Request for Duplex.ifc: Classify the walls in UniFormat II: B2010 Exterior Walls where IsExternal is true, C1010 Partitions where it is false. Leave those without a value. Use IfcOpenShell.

First a look at what the model holds.

```python
import ifcopenshell
import ifcopenshell.util.element

model = ifcopenshell.open("Duplex.ifc")
print(model.schema)
print("classifications:", [c.Name for c in model.by_type("IfcClassification")])
values = [ifcopenshell.util.element.get_pset(e, "Pset_WallCommon", "IsExternal") for e in model.by_type("IfcWall")]
for value in (True, False, None):
    print("IsExternal", value, values.count(value))
```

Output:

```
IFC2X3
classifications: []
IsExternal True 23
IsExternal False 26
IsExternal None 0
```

```python
import ifcopenshell
import ifcopenshell.api.classification
import ifcopenshell.util.element

model = ifcopenshell.open("Duplex.ifc")

# IFC2X3 requires Source and Edition and has no link from the project to the system.
system = model.create_entity("IfcClassification", Source="ASTM", Edition="E1557", Name="UniFormat II")

walls = model.by_type("IfcWall")
external = {e: ifcopenshell.util.element.get_pset(e, "Pset_WallCommon", "IsExternal") for e in walls}
for flag, code, name in ((True, "B2010", "Exterior Walls"), (False, "C1010", "Partitions")):
    products = [e for e in walls if external[e] is flag]
    ifcopenshell.api.classification.add_reference(
        model, products=products, classification=system, identification=code, name=name
    )
    print(code, len(products))

model.write("Duplex_edited.ifc")
```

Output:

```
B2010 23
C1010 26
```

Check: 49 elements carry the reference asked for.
